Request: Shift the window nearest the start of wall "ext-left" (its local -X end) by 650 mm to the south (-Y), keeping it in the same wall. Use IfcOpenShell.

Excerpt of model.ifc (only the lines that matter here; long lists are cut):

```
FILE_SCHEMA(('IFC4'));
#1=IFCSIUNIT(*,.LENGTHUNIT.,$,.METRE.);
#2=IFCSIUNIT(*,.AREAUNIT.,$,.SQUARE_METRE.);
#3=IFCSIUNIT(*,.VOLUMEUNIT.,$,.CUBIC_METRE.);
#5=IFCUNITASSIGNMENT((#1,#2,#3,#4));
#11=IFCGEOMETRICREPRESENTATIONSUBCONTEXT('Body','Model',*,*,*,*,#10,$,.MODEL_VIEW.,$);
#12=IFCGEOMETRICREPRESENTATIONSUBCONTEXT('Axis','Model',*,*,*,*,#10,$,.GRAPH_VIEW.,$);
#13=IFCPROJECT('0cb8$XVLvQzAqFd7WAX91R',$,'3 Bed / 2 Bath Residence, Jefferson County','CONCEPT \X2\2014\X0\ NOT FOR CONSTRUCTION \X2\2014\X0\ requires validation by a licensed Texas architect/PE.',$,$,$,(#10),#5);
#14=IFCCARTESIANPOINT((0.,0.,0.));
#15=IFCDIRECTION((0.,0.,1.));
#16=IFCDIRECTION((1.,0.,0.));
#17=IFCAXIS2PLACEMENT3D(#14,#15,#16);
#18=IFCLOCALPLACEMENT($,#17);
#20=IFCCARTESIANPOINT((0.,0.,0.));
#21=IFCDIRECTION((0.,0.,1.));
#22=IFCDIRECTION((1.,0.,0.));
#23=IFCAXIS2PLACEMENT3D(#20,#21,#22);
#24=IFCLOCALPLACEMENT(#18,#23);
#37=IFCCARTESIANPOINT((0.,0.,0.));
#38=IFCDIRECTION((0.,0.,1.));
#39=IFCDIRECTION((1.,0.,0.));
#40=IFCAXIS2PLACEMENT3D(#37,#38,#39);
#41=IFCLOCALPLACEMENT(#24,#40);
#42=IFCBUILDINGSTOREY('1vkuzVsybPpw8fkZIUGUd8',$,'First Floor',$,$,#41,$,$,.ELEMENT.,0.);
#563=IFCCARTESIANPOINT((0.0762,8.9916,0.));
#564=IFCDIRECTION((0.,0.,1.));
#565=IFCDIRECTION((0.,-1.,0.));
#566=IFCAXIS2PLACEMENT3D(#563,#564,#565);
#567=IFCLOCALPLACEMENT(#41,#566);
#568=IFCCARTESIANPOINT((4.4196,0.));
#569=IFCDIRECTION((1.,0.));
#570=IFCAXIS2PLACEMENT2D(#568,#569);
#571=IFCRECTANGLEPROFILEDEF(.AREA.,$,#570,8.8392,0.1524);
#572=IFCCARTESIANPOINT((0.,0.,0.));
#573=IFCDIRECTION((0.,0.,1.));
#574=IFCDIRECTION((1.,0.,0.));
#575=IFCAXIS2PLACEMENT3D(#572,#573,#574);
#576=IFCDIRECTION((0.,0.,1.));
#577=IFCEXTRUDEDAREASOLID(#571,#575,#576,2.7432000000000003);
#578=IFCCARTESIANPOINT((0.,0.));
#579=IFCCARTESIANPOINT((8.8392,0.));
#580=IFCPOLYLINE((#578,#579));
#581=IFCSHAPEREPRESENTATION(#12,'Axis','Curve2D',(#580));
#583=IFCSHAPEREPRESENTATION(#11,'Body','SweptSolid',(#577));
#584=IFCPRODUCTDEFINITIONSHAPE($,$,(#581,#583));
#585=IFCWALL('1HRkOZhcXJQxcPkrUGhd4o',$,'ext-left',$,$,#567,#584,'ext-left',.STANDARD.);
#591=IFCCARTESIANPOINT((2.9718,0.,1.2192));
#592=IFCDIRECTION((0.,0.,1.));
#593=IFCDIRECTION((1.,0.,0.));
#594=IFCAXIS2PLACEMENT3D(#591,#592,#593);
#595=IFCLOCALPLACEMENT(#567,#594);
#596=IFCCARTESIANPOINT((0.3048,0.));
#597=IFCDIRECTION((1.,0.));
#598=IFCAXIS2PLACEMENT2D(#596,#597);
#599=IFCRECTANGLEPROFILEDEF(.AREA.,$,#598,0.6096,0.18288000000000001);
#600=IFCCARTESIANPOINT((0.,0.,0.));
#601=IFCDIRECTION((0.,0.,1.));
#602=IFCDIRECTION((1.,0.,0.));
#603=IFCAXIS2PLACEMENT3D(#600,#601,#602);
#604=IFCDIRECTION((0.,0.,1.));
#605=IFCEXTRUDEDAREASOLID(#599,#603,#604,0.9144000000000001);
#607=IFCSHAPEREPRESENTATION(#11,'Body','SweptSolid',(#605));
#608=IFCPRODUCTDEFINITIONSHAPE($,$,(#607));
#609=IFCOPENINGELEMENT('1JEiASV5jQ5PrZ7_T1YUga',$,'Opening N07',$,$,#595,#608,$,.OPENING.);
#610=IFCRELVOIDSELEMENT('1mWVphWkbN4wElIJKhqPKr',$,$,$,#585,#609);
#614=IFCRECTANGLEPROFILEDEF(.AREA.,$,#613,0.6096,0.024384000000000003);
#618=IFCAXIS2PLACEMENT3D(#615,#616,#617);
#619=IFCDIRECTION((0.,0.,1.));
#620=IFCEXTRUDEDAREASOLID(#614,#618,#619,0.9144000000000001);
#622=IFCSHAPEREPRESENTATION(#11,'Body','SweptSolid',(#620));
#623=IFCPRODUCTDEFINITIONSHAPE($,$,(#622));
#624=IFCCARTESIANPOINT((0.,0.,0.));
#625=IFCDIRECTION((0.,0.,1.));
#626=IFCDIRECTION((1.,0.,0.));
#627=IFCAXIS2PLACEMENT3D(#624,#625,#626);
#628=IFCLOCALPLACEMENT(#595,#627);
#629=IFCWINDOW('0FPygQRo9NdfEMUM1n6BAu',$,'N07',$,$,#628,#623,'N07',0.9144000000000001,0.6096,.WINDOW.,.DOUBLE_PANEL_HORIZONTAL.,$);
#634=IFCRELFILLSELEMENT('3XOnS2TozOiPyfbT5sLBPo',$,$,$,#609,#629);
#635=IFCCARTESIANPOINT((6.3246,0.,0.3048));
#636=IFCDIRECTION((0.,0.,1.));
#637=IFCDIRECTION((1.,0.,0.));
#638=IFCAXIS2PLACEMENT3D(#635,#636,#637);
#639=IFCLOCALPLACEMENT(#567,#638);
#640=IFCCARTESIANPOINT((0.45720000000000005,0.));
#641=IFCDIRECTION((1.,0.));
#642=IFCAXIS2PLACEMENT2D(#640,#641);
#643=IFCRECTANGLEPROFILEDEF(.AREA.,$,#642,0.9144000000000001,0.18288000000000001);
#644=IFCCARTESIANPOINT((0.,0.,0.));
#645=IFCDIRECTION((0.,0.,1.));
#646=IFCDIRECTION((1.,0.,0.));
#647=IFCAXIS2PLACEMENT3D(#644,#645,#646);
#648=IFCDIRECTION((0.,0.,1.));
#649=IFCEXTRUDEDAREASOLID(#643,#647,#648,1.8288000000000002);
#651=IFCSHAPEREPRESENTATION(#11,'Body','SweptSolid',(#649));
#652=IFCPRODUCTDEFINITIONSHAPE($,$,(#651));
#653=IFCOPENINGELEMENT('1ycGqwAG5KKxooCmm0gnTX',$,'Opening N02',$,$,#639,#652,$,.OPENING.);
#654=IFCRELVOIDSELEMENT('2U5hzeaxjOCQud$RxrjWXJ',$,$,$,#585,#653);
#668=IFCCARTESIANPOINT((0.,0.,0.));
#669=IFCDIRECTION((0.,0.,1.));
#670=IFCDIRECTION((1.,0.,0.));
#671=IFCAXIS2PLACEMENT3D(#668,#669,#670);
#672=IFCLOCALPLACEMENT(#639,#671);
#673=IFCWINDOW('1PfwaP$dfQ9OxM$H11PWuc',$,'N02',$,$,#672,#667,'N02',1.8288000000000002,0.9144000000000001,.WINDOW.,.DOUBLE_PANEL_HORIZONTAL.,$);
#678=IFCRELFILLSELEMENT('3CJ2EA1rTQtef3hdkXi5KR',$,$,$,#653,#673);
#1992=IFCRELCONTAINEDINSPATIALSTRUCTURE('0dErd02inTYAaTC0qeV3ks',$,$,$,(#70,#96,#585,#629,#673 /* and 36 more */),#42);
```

```python
import ifcopenshell
import ifcopenshell.api.geometry
import ifcopenshell.util.placement
import ifcopenshell.util.unit

model = ifcopenshell.open("model.ifc")
unit_scale = ifcopenshell.util.unit.calculate_unit_scale(model)

window = model.by_guid("0FPygQRo9NdfEMUM1n6BAu")
opening = window.FillsVoids[0].RelatingOpeningElement
wall = opening.VoidsElements[0].RelatingBuildingElement

wall_matrix = ifcopenshell.util.placement.get_local_placement(wall.ObjectPlacement)
shift = wall_matrix[:3, 0] * 0.65 / unit_scale
before = ifcopenshell.util.placement.get_local_placement(window.ObjectPlacement)[:3, 3].copy()

# The window is placed relative to its opening, so it follows when the opening moves.
matrix = ifcopenshell.util.placement.get_local_placement(opening.ObjectPlacement)
matrix[:3, 3] += shift
ifcopenshell.api.geometry.edit_object_placement(
    model, product=opening, matrix=matrix, is_si=False, should_transform_children=True
)

after = ifcopenshell.util.placement.get_local_placement(window.ObjectPlacement)[:3, 3]
print("window moved by", (after - before).round(3) + 0.0)

model.write("model-out.ifc")
```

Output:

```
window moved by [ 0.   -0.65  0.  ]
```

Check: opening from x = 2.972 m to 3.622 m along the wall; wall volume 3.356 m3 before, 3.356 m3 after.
